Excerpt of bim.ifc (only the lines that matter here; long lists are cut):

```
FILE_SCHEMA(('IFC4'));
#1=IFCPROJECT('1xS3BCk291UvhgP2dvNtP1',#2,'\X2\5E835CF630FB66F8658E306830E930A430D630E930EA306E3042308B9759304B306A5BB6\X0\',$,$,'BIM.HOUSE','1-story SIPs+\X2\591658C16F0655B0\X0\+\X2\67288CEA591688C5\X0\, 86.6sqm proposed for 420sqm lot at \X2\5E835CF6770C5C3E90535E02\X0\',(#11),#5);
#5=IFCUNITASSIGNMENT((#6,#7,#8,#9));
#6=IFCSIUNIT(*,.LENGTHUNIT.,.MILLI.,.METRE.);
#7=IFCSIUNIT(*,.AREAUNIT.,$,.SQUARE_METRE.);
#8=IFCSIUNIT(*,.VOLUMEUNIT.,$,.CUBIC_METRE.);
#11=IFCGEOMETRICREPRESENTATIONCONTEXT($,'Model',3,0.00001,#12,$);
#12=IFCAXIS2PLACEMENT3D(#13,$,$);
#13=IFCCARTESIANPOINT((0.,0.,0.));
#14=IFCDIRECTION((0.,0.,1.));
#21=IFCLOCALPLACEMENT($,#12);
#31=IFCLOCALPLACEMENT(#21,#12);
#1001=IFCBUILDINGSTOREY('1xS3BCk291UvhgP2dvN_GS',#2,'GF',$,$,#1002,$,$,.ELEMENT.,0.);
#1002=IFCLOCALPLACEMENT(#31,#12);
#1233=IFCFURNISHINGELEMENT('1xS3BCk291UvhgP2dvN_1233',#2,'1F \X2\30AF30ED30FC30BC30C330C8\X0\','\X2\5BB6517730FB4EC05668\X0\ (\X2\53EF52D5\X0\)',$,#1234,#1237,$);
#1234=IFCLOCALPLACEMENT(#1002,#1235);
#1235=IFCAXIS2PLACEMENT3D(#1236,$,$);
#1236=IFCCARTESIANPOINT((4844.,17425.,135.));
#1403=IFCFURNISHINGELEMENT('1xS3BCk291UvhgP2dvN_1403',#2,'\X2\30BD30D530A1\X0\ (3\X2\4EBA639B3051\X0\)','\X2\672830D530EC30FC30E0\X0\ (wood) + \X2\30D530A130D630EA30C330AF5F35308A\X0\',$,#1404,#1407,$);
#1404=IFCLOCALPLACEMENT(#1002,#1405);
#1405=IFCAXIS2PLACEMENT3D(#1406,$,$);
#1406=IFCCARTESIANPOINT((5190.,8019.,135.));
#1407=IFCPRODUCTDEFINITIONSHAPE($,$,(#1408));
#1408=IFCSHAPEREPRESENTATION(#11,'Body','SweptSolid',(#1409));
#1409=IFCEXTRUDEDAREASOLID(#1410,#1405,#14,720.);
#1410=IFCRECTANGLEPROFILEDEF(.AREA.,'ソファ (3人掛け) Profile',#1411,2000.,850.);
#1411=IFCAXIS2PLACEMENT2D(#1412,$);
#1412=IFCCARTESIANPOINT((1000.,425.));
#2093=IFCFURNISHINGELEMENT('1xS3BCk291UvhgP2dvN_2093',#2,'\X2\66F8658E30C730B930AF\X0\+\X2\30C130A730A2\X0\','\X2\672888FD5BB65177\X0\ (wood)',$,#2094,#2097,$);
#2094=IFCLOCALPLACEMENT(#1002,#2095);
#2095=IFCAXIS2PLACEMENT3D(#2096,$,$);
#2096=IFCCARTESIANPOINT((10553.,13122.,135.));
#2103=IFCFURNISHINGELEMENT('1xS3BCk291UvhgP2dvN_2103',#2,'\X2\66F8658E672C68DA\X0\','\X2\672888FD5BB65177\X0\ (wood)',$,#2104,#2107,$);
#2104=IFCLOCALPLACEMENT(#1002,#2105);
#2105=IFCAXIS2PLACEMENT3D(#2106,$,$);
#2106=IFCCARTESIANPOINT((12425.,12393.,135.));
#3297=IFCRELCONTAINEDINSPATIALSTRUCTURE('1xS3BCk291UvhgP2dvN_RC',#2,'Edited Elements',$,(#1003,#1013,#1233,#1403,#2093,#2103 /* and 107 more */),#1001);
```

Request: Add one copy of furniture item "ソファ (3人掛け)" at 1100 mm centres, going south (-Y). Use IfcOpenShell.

```python
import numpy as np
import ifcopenshell
import ifcopenshell.api.geometry
import ifcopenshell.api.root
import ifcopenshell.util.element
import ifcopenshell.util.placement
import ifcopenshell.util.unit

model = ifcopenshell.open("bim.ifc")
unit_scale = ifcopenshell.util.unit.calculate_unit_scale(model)


def reuse_history(source, copy):
    """copy_class also copies each property set's owner history, people and application; keep the originals."""
    for rel in copy.IsDefinedBy:
        if rel.is_a("IfcRelDefinesByProperties") and (history := rel.RelatingPropertyDefinition.OwnerHistory):
            rel.RelatingPropertyDefinition.OwnerHistory = source.OwnerHistory
            ifcopenshell.util.element.remove_deep2(model, history)


source = model.by_guid("1xS3BCk291UvhgP2dvN_1403")
base = ifcopenshell.util.placement.get_local_placement(source.ObjectPlacement)
step = np.array([0.0, -1.0, 0.0]) * 1.1 / unit_scale

for i in range(1, 2):
    copy = ifcopenshell.api.root.copy_class(model, product=source)
    copy.Representation = ifcopenshell.util.element.copy_deep(
        model, source.Representation, exclude=["IfcGeometricRepresentationContext", "IfcRepresentationMap"]
    )
    reuse_history(source, copy)
    matrix = base.copy()
    matrix[:3, 3] += i * step
    print("added at", matrix[:3, 3].round(3) + 0.0)
    ifcopenshell.api.geometry.edit_object_placement(model, product=copy, matrix=matrix, is_si=False)

model.write("bim_rev.ifc")
```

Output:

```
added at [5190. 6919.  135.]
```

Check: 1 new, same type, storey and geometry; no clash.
